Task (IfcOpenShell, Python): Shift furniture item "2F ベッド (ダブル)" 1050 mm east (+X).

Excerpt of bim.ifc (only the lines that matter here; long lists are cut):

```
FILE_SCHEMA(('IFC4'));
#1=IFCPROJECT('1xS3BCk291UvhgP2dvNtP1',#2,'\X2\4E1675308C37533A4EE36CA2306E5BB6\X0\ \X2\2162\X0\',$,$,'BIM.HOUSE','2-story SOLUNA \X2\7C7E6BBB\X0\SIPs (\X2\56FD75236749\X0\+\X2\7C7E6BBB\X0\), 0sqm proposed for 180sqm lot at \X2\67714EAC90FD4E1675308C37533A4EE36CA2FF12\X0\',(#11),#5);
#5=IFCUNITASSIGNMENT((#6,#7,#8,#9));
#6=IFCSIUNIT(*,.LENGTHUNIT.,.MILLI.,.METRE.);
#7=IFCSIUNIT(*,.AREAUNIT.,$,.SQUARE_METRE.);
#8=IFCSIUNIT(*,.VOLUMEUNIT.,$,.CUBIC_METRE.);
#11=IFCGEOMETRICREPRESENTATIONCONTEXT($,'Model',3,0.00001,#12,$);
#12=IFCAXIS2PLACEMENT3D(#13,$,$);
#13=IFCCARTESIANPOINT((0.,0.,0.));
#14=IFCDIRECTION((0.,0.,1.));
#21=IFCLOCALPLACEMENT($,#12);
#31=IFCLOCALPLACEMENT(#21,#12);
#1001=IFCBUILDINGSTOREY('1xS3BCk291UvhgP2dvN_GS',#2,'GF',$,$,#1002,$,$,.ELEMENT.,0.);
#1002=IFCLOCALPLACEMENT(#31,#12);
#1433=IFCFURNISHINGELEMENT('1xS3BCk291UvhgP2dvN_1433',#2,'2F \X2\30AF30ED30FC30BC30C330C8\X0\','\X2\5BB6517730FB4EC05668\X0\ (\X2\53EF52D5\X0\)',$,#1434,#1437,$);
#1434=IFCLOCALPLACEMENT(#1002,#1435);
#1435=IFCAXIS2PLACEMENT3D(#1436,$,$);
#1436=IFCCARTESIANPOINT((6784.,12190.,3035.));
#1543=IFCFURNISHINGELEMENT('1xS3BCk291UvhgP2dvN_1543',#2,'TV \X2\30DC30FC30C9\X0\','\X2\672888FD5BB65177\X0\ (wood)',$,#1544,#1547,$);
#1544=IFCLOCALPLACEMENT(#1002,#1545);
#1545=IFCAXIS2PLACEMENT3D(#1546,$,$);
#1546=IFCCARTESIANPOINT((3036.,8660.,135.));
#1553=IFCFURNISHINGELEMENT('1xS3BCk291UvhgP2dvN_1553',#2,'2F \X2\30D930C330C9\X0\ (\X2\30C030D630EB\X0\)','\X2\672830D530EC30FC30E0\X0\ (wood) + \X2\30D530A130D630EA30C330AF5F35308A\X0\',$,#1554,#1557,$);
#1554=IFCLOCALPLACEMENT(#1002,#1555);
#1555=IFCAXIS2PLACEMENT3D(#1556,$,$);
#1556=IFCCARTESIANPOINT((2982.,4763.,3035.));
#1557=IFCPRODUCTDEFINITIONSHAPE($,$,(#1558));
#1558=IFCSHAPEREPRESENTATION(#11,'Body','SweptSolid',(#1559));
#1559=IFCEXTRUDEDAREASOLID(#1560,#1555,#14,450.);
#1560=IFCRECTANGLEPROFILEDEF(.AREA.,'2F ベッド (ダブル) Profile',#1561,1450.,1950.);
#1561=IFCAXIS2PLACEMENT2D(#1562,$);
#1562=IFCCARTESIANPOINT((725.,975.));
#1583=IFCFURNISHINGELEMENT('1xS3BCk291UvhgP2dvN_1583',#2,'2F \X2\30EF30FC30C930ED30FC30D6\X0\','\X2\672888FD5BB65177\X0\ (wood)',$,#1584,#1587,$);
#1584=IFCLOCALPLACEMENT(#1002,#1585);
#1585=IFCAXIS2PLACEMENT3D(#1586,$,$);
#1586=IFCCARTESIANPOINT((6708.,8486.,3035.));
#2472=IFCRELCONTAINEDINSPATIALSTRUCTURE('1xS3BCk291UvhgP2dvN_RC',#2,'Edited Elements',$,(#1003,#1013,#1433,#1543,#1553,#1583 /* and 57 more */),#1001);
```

```python
import ifcopenshell
import ifcopenshell.api.geometry
import ifcopenshell.util.placement
import ifcopenshell.util.unit

model = ifcopenshell.open("bim.ifc")
unit_scale = ifcopenshell.util.unit.calculate_unit_scale(model)

item = model.by_id(1553)
matrix = ifcopenshell.util.placement.get_local_placement(item.ObjectPlacement)
matrix[0, 3] += 1.05 / unit_scale
ifcopenshell.api.geometry.edit_object_placement(model, product=item, matrix=matrix, is_si=False)

print(ifcopenshell.util.placement.get_local_placement(item.ObjectPlacement).round(3) + 0.0)

model.write("bim_rev.ifc")
```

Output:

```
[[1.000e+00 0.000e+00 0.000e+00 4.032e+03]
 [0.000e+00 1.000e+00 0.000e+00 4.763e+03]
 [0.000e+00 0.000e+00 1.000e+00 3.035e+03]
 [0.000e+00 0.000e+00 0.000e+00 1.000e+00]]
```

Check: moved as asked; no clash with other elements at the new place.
